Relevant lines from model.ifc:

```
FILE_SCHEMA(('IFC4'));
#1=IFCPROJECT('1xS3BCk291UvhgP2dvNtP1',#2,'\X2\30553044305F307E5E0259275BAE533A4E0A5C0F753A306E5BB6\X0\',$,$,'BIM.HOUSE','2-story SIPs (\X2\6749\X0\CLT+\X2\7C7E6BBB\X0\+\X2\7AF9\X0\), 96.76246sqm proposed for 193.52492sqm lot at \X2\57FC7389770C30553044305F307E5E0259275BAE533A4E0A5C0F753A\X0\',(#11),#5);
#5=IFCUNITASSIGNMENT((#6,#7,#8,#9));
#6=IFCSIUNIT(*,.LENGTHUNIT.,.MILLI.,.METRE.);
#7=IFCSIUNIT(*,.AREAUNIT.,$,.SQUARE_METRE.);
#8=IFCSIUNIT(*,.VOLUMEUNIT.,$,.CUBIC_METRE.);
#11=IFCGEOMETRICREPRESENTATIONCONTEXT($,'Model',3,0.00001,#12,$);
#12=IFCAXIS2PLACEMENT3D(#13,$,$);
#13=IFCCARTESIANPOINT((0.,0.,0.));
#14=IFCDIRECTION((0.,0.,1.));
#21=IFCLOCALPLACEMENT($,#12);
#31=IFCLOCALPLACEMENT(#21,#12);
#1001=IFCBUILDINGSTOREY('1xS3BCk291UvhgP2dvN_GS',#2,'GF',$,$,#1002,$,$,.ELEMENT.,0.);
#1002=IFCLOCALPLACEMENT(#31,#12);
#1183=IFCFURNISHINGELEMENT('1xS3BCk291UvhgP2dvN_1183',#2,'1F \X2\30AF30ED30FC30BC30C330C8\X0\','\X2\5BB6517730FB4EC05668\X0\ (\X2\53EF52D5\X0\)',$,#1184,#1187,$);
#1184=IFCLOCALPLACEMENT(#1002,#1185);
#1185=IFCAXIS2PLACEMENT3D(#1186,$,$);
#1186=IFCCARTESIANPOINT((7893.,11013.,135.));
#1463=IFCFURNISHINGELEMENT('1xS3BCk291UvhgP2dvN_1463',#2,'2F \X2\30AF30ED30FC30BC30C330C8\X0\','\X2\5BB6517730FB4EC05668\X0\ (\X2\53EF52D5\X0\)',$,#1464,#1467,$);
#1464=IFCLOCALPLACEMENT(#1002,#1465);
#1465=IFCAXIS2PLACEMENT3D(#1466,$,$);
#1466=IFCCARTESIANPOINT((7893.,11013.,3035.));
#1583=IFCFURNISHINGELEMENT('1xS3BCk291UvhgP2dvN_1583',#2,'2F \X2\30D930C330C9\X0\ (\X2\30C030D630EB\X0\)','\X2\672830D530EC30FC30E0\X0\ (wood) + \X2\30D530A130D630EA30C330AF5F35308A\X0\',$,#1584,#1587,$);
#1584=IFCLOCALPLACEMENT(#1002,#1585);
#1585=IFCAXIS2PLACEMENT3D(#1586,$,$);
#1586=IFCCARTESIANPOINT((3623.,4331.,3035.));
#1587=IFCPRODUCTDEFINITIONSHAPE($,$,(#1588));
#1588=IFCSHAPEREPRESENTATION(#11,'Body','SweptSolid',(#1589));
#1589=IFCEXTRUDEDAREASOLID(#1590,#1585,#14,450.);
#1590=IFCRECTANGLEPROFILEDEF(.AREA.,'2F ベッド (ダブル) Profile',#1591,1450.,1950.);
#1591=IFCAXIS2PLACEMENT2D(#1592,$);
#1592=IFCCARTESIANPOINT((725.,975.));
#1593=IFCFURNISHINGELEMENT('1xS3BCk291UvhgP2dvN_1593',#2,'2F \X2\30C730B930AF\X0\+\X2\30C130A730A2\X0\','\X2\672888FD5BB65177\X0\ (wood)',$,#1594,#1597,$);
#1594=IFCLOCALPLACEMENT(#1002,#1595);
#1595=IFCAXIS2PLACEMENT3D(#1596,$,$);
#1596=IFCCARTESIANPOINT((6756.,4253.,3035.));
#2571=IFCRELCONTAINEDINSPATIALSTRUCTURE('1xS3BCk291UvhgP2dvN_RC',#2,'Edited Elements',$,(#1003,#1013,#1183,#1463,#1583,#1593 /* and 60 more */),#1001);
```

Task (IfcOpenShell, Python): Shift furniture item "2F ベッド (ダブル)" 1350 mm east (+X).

```python
import ifcopenshell
import ifcopenshell.api.geometry
import ifcopenshell.util.placement
import ifcopenshell.util.unit

model = ifcopenshell.open("model.ifc")
unit_scale = ifcopenshell.util.unit.calculate_unit_scale(model)

item = model.by_id(1583)
matrix = ifcopenshell.util.placement.get_local_placement(item.ObjectPlacement)
matrix[0, 3] += 1.35 / unit_scale
ifcopenshell.api.geometry.edit_object_placement(model, product=item, matrix=matrix, is_si=False)

print(ifcopenshell.util.placement.get_local_placement(item.ObjectPlacement).round(3) + 0.0)

model.write("model_rev.ifc")
```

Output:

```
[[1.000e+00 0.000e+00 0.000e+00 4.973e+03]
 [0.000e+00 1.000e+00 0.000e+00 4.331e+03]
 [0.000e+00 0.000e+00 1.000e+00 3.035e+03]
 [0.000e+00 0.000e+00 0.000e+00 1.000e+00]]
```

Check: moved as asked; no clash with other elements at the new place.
